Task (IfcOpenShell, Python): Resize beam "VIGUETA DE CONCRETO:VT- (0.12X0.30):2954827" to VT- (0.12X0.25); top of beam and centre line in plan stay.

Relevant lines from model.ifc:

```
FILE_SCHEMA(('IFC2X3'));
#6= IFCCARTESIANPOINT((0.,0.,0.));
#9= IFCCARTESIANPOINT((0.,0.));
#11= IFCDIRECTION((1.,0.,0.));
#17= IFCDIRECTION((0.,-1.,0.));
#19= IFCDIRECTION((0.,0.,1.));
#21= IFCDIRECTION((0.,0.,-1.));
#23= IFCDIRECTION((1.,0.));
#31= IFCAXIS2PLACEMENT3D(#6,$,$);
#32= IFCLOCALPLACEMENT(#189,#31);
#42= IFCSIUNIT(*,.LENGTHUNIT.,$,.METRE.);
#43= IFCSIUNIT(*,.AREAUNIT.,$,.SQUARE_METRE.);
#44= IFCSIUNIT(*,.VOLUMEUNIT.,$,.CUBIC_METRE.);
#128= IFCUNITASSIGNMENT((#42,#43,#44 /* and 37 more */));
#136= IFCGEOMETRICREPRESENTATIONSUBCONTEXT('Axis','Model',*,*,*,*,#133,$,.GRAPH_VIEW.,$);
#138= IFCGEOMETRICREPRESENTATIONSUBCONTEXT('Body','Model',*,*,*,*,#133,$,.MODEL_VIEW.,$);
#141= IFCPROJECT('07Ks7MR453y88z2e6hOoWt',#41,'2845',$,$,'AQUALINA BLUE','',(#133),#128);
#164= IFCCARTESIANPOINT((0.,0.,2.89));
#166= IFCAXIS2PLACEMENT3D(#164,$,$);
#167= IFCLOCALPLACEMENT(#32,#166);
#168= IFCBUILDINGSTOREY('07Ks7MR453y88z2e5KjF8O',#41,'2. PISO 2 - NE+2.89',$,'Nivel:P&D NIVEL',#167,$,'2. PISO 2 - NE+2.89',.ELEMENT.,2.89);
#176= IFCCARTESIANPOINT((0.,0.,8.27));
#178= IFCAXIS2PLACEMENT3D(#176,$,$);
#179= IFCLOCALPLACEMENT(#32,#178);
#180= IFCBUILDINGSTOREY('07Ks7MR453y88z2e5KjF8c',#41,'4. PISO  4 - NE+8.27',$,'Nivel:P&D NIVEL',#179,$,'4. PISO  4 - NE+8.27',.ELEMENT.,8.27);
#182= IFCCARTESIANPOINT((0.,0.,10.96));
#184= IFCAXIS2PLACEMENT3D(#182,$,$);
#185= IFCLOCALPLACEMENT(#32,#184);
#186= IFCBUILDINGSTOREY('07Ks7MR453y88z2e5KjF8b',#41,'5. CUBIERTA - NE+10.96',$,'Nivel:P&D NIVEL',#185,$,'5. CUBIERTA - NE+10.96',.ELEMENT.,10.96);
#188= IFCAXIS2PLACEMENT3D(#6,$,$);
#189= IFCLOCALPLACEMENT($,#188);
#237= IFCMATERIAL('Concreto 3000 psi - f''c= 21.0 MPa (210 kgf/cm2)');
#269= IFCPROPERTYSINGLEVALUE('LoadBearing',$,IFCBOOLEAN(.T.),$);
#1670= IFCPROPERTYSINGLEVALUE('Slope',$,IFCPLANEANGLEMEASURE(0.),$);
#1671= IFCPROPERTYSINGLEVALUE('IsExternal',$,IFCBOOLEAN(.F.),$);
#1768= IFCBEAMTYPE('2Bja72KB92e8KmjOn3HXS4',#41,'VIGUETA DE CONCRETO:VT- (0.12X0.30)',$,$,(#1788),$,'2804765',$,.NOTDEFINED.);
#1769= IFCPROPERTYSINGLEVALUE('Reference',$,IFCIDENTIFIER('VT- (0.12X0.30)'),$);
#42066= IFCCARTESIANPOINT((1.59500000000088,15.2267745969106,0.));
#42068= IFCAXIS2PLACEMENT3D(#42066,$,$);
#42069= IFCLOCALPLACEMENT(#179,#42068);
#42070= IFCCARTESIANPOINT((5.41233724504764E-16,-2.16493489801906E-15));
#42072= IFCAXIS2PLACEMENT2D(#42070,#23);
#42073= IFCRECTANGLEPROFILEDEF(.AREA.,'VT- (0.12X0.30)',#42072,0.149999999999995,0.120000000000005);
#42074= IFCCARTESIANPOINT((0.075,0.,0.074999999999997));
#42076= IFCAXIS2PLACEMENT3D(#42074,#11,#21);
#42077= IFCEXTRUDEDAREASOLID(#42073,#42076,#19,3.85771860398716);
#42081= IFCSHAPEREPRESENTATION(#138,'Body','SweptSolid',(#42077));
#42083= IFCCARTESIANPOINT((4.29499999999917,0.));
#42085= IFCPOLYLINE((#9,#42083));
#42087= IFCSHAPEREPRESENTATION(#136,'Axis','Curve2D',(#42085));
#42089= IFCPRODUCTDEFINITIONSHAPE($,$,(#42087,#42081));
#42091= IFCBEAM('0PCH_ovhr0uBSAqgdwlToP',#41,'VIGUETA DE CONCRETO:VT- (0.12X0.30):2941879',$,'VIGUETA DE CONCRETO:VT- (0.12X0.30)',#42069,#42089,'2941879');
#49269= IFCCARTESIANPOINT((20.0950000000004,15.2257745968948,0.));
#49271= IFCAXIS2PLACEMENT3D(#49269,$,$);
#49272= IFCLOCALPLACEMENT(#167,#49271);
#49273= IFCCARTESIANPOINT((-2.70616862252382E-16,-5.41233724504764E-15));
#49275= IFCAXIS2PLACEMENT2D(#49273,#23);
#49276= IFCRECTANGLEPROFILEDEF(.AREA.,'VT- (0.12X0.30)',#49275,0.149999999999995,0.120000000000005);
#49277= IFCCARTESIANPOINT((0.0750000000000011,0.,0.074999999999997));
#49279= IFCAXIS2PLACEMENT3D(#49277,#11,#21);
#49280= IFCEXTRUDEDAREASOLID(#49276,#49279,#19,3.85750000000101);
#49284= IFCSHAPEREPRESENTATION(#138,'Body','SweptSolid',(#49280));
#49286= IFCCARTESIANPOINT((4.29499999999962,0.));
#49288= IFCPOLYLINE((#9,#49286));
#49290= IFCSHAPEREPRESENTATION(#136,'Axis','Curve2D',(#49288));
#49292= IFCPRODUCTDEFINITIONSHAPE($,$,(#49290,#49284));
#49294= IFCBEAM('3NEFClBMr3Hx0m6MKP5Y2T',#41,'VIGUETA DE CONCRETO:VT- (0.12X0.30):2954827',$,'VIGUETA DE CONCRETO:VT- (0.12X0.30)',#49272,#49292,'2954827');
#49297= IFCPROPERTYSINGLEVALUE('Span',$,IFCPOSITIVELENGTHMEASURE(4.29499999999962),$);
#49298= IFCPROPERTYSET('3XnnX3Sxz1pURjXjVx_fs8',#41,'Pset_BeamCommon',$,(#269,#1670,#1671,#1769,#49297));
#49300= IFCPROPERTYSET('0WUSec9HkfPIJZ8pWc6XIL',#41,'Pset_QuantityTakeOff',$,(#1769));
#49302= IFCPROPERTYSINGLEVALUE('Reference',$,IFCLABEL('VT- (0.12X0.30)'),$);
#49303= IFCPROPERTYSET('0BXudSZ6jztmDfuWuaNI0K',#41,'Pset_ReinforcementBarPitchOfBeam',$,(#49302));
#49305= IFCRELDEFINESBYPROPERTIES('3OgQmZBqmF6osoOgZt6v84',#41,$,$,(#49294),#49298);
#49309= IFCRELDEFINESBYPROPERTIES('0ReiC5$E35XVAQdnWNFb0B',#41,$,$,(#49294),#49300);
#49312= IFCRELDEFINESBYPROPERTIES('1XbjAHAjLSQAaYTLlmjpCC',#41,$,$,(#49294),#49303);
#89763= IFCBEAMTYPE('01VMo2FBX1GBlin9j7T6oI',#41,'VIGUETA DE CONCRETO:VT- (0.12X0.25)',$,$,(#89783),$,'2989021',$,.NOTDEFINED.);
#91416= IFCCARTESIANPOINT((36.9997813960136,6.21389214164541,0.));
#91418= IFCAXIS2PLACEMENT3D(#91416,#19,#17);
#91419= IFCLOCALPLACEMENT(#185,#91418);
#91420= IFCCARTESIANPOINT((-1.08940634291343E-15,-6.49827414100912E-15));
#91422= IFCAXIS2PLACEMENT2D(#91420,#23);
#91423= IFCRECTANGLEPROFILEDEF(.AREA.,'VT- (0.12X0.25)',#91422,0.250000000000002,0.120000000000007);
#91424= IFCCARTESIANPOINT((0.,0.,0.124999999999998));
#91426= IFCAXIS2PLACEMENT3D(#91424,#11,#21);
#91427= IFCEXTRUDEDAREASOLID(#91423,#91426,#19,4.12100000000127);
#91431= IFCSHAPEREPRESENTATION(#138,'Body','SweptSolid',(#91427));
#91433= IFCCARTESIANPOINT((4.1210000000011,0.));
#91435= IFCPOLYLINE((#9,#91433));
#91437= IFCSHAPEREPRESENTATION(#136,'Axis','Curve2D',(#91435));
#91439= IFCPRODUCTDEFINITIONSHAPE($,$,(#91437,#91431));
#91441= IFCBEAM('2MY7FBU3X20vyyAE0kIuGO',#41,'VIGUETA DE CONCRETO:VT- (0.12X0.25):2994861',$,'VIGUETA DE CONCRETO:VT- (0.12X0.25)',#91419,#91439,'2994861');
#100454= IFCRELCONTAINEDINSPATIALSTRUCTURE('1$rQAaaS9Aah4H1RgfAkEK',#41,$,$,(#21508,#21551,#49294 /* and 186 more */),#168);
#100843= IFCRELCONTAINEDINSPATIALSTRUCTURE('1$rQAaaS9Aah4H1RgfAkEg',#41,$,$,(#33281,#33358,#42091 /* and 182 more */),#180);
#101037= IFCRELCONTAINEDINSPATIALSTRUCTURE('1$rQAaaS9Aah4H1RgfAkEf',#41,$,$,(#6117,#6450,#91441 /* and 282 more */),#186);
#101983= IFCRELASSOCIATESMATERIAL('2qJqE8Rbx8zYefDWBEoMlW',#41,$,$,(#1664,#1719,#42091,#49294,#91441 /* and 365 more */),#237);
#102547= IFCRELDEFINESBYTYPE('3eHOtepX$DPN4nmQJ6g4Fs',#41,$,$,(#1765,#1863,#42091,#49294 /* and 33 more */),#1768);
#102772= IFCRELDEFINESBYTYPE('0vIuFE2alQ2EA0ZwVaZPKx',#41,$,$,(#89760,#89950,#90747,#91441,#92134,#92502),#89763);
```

```python
import ifcopenshell
import ifcopenshell.api.pset
import ifcopenshell.api.type
import ifcopenshell.util.element
import ifcopenshell.util.representation

model = ifcopenshell.open("model.ifc")

member = model.by_guid("3NEFClBMr3Hx0m6MKP5Y2T")
source = next(p for p in model.by_type("IfcRectangleProfileDef") if p.ProfileName == "VT- (0.12X0.25)")

body = ifcopenshell.util.representation.get_representation(member, "Model", "Body")
solid = body.Items[0]
old_profile = solid.SweptArea

# Copy the section's sizes but keep this member's own profile position.
profile = ifcopenshell.util.element.copy(model, source)
# Profiles are centred, so shift by half the change in depth to hold the top.
shift = (old_profile.XDim - profile.XDim) / 2
x, y = old_profile.Position.Location.Coordinates
up = (-1.0, 0.0)  # upwards, in the solid's own plane
location = model.createIfcCartesianPoint((x + up[0] * shift, y + up[1] * shift))
profile.Position = model.createIfcAxis2Placement2D(location, old_profile.Position.RefDirection)
solid.SweptArea = profile
if not model.get_total_inverses(old_profile):
    ifcopenshell.util.element.remove_deep2(model, old_profile)

new_type = model.by_guid("01VMo2FBX1GBlin9j7T6oI")
ifcopenshell.api.type.assign_type(
    model, related_objects=[member], relating_type=new_type, should_map_representations=False
)
member.Name = member.Name.replace("VT- (0.12X0.30)", "VT- (0.12X0.25)")
member.ObjectType = "VIGUETA DE CONCRETO:VT- (0.12X0.25)"
pset = model.by_id(ifcopenshell.util.element.get_pset(member, "Pset_BeamCommon", should_inherit=False)["id"])
ifcopenshell.api.pset.edit_pset(model, pset=pset, properties={"Reference": "VT- (0.12X0.25)"})
pset = model.by_id(ifcopenshell.util.element.get_pset(member, "Pset_QuantityTakeOff", should_inherit=False)["id"])
ifcopenshell.api.pset.edit_pset(model, pset=pset, properties={"Reference": "VT- (0.12X0.25)"})
pset = model.by_id(ifcopenshell.util.element.get_pset(member, "Pset_ReinforcementBarPitchOfBeam", should_inherit=False)["id"])
ifcopenshell.api.pset.edit_pset(model, pset=pset, properties={"Reference": "VT- (0.12X0.25)"})

print(solid.SweptArea)

model.write("model_updated.ifc")
```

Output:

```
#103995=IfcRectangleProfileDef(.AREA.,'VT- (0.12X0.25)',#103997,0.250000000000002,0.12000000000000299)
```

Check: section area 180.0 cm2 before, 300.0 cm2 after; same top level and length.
